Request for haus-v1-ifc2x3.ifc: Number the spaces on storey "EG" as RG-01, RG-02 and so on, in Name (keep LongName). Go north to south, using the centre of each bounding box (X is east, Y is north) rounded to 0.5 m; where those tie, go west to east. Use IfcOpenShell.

First a look at what the model holds.

```python
import ifcopenshell
import ifcopenshell.util.element
import ifcopenshell.util.placement

model = ifcopenshell.open("haus-v1-ifc2x3.ifc")
print(model.schema)
storey = next(s for s in model.by_type("IfcBuildingStorey") if s.Name == "EG")
spaces = [e for e in ifcopenshell.util.element.get_decomposition(storey) if e.is_a("IfcSpace")]
for e in sorted(spaces, key=lambda e: e.id()):
    origin = ifcopenshell.util.placement.get_local_placement(e.ObjectPlacement)[:3, 3]
    print(e.id(), e.Name, e.LongName, origin.round(2) + 0.0, sep=" | ")
```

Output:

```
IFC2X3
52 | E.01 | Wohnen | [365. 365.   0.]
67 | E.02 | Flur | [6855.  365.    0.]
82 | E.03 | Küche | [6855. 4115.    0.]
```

```python
import ifcopenshell
import ifcopenshell.geom
import ifcopenshell.util.element
import ifcopenshell.util.shape

model = ifcopenshell.open("haus-v1-ifc2x3.ifc")
settings = ifcopenshell.geom.settings()
settings.set("use-world-coords", True)


def centre(element):
    shape = ifcopenshell.geom.create_shape(settings, element)
    return ifcopenshell.util.shape.get_bbox_centroid(shape.geometry)


storey = next(s for s in model.by_type("IfcBuildingStorey") if s.Name == "EG")
spaces = [e for e in ifcopenshell.util.element.get_decomposition(storey) if e.is_a("IfcSpace")]

# Insertion points can sit at a corner or the storey origin, so sort by the geometry (in metres).
centres = {e: centre(e) for e in spaces}
spaces.sort(key=lambda e: (-round(centres[e][1] / 0.5), centres[e][0]))

for i, e in enumerate(spaces, start=1):
    number = f"RG-{i:02d}"
    e.Name = number
    print(e.id(), number)

model.write("haus-v1-ifc2x3-out.ifc")
```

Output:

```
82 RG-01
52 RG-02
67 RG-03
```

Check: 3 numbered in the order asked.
